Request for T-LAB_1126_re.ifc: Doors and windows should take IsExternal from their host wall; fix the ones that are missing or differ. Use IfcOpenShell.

First a look at what the model holds.

```python
import ifcopenshell
import ifcopenshell.util.element

model = ifcopenshell.open("T-LAB_1126_re.ifc")
print(model.schema)
seen = {}
for e in model.by_type("IfcDoor") + model.by_type("IfcWindow"):
    if not e.FillsVoids:
        continue
    host = e.FillsVoids[0].RelatingOpeningElement.VoidsElements[0].RelatingBuildingElement
    own = ifcopenshell.util.element.get_pset(e, f"Pset_{e.is_a()[3:].removesuffix('StandardCase')}Common", "IsExternal")
    wall = ifcopenshell.util.element.get_pset(host, "Pset_WallCommon", "IsExternal")
    seen[e.is_a(), own, wall] = seen.get((e.is_a(), own, wall), 0) + 1
for (cls, own, wall), count in sorted(seen.items(), key=str):
    print(count, cls, "IsExternal:", own, "| host wall:", wall)
```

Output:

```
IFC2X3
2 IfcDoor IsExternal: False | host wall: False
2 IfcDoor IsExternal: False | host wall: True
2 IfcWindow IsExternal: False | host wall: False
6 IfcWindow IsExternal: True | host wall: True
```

```python
import ifcopenshell
import ifcopenshell.api.pset
import ifcopenshell.util.element

model = ifcopenshell.open("T-LAB_1126_re.ifc")

count = 0
for ifc_class, pset_name in (("IfcDoor", "Pset_DoorCommon"), ("IfcWindow", "Pset_WindowCommon")):
    for e in model.by_type(ifc_class):
        if not e.FillsVoids:
            continue
        host = e.FillsVoids[0].RelatingOpeningElement.VoidsElements[0].RelatingBuildingElement
        external = ifcopenshell.util.element.get_pset(host, "Pset_WallCommon", "IsExternal")
        if external is None or ifcopenshell.util.element.get_pset(e, pset_name, "IsExternal") == external:
            continue
        pset = ifcopenshell.api.pset.add_pset(model, product=e, name=pset_name)
        ifcopenshell.api.pset.edit_pset(model, pset=pset, properties={"IsExternal": external})
        count += 1

print(count, "updated")

model.write("T-LAB_1126_re_updated.ifc")
```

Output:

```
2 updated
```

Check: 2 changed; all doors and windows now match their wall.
